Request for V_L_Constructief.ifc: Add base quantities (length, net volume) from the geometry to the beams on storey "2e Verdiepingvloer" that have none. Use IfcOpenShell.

First a look at what the model holds.

```python
import ifcopenshell
import ifcopenshell.util.element
import ifcopenshell.util.unit

model = ifcopenshell.open("V_L_Constructief.ifc")
print(model.schema)
for unit_type in ("LENGTHUNIT", "AREAUNIT", "VOLUMEUNIT"):
    print(unit_type, ifcopenshell.util.unit.calculate_unit_scale(model, unit_type))
storey = next(s for s in model.by_type("IfcBuildingStorey") if s.Name == "2e Verdiepingvloer")
beams = [e for e in ifcopenshell.util.element.get_decomposition(storey) if e.is_a("IfcBeam")]
for e in sorted(beams, key=lambda e: e.id()):
    print(e.id(), e.is_a(), e.Name, list(ifcopenshell.util.element.get_psets(e, qtos_only=True)), sep=" | ")
```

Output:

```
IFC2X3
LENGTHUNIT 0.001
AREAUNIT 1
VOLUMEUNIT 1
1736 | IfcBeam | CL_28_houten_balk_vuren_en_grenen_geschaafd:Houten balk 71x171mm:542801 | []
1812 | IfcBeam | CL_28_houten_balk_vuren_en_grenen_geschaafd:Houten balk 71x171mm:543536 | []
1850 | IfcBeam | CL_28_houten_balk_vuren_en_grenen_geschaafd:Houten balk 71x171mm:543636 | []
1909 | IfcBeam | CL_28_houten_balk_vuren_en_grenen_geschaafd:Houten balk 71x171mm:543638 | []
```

```python
import ifcopenshell
import ifcopenshell.api.pset
import ifcopenshell.geom
import ifcopenshell.util.element
import ifcopenshell.util.shape
import ifcopenshell.util.unit

model = ifcopenshell.open("V_L_Constructief.ifc")
unit_scale = ifcopenshell.util.unit.calculate_unit_scale(model)
volume_scale = ifcopenshell.util.unit.calculate_unit_scale(model, "VOLUMEUNIT")
settings = ifcopenshell.geom.settings()

storey = next(s for s in model.by_type("IfcBuildingStorey") if s.Name == "2e Verdiepingvloer")
beams = [e for e in ifcopenshell.util.element.get_decomposition(storey) if e.is_a("IfcBeam")]

for e in sorted(beams, key=lambda e: e.id()):
    if ifcopenshell.util.element.get_psets(e, qtos_only=True, should_inherit=False):
        continue
    # Geometry comes back in metres, in the element's own axes.
    shape = ifcopenshell.geom.create_shape(settings, e)
    values = {
        "Length": ifcopenshell.util.shape.get_max_xyz(shape.geometry) / unit_scale,
        "NetVolume": ifcopenshell.util.shape.get_volume(shape.geometry) / volume_scale,
    }
    qto = ifcopenshell.api.pset.add_qto(model, product=e, name="BaseQuantities")
    ifcopenshell.api.pset.edit_qto(model, qto=qto, properties=values)
    print(e.id(), {k: round(v, 3) for k, v in values.items()})

model.write("V_L_Constructief_v2.ifc")
```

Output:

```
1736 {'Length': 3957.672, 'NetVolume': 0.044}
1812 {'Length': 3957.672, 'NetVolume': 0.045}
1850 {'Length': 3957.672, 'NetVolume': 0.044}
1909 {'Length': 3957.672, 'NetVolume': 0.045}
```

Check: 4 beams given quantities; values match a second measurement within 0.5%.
